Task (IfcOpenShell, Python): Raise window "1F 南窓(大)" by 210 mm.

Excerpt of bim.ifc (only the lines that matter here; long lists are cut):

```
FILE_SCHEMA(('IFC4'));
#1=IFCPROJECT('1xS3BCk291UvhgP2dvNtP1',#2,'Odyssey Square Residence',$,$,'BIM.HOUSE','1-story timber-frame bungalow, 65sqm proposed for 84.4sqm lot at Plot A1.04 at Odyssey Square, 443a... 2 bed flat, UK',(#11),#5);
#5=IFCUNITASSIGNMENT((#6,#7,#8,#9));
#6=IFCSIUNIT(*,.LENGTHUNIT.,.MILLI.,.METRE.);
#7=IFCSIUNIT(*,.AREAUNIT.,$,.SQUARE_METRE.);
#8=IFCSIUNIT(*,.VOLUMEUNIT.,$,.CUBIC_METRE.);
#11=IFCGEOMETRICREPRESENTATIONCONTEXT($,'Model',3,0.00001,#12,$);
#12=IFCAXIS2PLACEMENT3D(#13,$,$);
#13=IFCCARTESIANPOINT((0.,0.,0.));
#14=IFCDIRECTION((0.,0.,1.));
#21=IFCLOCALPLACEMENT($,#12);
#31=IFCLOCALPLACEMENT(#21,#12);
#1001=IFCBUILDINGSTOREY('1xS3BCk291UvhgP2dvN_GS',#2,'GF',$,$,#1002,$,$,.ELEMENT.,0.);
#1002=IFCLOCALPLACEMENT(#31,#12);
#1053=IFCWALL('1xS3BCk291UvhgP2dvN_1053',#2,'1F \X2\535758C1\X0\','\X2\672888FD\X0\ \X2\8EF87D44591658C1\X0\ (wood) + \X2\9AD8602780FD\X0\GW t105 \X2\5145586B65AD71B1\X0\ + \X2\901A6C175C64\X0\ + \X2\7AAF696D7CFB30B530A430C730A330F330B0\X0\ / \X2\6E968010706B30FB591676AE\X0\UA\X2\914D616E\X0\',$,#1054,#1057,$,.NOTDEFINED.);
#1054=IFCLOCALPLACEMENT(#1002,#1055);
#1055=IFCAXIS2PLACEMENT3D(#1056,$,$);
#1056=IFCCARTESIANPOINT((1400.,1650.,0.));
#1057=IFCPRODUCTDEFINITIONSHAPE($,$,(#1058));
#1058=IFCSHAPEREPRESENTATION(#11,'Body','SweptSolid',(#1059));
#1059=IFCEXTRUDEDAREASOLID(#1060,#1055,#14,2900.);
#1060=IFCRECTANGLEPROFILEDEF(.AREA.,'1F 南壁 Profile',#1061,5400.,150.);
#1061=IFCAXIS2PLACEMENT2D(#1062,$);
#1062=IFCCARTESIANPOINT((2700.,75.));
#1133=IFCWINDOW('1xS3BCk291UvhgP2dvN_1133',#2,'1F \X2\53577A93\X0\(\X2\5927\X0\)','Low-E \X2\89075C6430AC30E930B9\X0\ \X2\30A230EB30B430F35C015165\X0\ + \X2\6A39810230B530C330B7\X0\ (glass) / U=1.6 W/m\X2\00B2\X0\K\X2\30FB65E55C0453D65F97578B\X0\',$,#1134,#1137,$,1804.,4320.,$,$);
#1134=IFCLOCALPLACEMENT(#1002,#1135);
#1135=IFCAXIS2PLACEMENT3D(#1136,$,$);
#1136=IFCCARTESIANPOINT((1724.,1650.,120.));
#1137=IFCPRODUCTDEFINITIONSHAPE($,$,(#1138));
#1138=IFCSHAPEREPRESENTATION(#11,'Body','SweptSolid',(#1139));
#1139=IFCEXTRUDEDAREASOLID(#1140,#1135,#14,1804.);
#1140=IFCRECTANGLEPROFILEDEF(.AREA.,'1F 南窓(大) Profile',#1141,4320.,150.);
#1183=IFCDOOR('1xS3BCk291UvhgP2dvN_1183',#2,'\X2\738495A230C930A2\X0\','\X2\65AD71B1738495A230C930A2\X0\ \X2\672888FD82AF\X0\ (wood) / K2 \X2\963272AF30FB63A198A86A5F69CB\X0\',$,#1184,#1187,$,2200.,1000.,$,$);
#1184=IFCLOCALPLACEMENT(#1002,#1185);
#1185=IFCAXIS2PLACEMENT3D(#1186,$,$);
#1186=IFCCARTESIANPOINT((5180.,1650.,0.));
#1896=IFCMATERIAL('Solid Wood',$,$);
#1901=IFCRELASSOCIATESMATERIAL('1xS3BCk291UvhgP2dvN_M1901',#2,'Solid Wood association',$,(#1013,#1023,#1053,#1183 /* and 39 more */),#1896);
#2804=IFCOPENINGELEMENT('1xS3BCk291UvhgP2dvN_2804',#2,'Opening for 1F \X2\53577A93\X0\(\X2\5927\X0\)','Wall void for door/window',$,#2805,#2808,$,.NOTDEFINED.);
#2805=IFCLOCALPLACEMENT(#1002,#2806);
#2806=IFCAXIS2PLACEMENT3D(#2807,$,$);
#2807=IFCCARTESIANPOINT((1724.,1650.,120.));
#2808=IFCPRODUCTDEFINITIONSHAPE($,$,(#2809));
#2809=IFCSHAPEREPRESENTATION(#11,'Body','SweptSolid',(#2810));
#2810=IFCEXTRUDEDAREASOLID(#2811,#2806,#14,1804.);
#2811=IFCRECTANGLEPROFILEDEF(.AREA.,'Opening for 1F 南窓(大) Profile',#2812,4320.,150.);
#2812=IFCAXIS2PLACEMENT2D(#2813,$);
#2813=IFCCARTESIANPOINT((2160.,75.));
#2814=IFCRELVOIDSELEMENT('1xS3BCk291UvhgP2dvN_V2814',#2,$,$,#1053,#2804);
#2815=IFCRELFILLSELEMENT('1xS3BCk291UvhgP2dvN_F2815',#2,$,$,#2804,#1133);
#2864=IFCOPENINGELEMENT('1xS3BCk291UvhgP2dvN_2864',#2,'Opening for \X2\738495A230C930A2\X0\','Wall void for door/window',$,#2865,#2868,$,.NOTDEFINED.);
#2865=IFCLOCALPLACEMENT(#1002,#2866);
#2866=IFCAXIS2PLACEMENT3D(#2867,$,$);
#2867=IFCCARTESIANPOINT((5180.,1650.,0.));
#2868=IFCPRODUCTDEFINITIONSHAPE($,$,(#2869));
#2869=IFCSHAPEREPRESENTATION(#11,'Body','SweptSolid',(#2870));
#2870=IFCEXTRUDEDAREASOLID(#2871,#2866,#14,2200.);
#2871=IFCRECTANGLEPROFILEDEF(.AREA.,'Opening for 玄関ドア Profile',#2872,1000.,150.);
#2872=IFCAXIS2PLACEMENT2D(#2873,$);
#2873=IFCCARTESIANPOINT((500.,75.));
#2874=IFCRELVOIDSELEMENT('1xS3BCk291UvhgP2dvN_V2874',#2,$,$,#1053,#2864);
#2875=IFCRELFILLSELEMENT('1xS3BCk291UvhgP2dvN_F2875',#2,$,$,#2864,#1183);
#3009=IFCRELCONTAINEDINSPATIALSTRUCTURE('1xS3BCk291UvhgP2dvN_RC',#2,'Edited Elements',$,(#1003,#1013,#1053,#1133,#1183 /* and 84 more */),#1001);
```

```python
import numpy as np
import ifcopenshell
import ifcopenshell.api.geometry
import ifcopenshell.util.placement
import ifcopenshell.util.unit

model = ifcopenshell.open("bim.ifc")
unit_scale = ifcopenshell.util.unit.calculate_unit_scale(model)

window = model.by_guid("1xS3BCk291UvhgP2dvN_1133")
opening = window.FillsVoids[0].RelatingOpeningElement
dz = 0.21 / unit_scale

shift = np.array([0.0, 0.0, dz])
# The window is not placed relative to its opening, so move both.
for product in (opening, window):
    matrix = ifcopenshell.util.placement.get_local_placement(product.ObjectPlacement)
    matrix[:3, 3] += shift
    ifcopenshell.api.geometry.edit_object_placement(model, product=product, matrix=matrix, is_si=False)

print(f"moved by {dz * unit_scale:+.3f} m")

model.write("bim-out.ifc")
```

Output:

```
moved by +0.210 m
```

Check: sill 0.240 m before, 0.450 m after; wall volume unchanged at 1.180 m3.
